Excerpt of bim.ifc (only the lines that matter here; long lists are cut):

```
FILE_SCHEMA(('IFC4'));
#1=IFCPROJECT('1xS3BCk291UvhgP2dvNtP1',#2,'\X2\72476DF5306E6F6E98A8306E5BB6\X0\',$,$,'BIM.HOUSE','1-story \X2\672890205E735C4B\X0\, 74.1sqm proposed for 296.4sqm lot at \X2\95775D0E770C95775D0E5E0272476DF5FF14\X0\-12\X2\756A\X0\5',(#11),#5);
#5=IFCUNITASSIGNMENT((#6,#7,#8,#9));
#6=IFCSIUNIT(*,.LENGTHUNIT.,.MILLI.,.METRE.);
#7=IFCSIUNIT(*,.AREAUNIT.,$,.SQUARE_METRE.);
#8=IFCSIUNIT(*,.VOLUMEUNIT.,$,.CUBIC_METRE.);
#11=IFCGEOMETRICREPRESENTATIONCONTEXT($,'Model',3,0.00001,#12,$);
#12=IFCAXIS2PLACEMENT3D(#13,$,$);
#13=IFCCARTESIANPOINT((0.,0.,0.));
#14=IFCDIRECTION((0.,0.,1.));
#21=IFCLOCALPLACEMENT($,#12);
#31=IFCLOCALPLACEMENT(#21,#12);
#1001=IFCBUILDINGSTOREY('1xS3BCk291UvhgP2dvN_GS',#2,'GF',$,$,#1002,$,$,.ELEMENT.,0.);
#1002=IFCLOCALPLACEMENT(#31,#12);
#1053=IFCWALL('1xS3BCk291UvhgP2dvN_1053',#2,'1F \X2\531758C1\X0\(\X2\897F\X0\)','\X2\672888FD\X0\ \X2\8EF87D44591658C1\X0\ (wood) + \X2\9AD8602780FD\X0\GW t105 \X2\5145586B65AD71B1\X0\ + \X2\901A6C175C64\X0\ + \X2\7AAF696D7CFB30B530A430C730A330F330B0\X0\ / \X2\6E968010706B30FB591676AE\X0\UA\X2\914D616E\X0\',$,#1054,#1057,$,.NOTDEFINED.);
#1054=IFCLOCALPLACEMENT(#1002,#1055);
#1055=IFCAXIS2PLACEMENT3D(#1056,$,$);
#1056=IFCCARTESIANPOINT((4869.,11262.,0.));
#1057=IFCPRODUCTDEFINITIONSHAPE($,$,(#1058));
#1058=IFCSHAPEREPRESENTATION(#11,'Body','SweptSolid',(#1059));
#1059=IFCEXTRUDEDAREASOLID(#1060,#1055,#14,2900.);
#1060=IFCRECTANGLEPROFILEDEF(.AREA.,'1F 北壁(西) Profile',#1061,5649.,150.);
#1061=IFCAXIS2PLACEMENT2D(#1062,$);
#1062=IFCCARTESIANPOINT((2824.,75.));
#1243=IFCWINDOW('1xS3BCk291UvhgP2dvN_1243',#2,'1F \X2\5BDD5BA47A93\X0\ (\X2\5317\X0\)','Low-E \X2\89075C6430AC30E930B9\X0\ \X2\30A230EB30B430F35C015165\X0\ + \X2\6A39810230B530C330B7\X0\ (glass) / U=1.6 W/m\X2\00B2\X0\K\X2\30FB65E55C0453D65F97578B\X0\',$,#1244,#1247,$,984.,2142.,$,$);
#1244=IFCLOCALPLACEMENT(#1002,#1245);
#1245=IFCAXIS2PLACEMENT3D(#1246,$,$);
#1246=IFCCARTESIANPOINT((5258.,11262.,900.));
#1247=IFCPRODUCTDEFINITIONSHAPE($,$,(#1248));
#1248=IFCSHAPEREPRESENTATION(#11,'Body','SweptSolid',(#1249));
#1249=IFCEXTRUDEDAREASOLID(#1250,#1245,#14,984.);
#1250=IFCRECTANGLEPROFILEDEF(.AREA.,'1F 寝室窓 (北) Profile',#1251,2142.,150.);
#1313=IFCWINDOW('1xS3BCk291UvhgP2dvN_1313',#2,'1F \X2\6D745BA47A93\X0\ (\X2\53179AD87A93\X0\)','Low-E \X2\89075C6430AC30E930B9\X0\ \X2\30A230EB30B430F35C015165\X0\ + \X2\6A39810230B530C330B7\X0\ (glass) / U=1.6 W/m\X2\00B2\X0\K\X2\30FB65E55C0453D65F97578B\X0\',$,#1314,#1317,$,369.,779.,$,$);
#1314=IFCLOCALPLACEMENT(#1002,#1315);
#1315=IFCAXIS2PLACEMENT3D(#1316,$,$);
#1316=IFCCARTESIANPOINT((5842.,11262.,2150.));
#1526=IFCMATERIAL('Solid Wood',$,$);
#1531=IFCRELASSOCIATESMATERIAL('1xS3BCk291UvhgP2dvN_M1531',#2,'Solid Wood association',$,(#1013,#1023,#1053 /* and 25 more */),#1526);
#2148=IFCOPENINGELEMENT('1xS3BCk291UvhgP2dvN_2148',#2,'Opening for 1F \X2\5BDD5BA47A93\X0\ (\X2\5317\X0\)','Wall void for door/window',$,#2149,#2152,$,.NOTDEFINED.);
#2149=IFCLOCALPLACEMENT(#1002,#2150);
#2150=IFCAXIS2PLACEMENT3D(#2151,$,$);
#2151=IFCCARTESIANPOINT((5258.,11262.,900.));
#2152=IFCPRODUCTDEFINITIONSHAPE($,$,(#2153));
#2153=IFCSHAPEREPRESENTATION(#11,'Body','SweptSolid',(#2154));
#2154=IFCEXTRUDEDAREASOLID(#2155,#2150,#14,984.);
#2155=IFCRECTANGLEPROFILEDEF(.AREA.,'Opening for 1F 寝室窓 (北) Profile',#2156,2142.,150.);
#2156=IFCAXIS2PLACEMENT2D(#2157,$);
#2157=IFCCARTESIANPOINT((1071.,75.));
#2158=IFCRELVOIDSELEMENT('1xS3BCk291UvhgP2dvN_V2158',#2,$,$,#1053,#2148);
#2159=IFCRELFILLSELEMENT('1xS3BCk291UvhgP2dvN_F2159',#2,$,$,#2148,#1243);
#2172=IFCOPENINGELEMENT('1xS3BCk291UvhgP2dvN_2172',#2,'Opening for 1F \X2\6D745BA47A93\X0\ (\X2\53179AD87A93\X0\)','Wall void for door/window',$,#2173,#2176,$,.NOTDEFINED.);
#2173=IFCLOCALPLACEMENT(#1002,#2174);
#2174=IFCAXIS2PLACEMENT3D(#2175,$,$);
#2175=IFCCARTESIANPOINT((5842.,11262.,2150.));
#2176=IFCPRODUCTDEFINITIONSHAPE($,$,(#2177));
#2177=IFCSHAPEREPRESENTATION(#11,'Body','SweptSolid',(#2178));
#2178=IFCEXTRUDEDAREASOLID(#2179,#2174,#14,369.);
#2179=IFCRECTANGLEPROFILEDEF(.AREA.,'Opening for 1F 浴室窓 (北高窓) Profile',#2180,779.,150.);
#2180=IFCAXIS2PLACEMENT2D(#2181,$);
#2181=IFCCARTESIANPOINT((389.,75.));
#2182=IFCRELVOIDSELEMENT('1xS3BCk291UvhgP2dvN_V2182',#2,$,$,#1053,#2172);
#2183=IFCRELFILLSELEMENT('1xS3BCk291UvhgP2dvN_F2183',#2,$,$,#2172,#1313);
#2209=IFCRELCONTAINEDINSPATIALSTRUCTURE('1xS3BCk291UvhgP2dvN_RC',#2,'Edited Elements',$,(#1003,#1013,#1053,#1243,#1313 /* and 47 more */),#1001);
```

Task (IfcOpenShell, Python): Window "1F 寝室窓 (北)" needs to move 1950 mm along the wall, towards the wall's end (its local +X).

```python
import ifcopenshell
import ifcopenshell.api.geometry
import ifcopenshell.util.placement
import ifcopenshell.util.unit

model = ifcopenshell.open("bim.ifc")
unit_scale = ifcopenshell.util.unit.calculate_unit_scale(model)

window = model.by_id(1243)
opening = window.FillsVoids[0].RelatingOpeningElement
wall = opening.VoidsElements[0].RelatingBuildingElement

wall_matrix = ifcopenshell.util.placement.get_local_placement(wall.ObjectPlacement)
shift = wall_matrix[:3, 0] * 1.95 / unit_scale
before = ifcopenshell.util.placement.get_local_placement(window.ObjectPlacement)[:3, 3].copy()

# The window is not placed relative to its opening, so move both.
for product in (opening, window):
    matrix = ifcopenshell.util.placement.get_local_placement(product.ObjectPlacement)
    matrix[:3, 3] += shift
    ifcopenshell.api.geometry.edit_object_placement(model, product=product, matrix=matrix, is_si=False)

after = ifcopenshell.util.placement.get_local_placement(window.ObjectPlacement)[:3, 3]
print("window moved by", (after - before).round(3) + 0.0)

model.write("bim_edited.ifc")
```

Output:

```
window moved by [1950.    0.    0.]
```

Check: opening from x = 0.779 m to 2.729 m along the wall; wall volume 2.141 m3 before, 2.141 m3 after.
